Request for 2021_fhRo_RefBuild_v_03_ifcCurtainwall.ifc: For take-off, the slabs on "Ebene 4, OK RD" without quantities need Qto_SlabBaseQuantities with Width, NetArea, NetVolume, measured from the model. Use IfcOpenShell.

First a look at what the model holds.

```python
import ifcopenshell
import ifcopenshell.util.element
import ifcopenshell.util.unit

model = ifcopenshell.open("2021_fhRo_RefBuild_v_03_ifcCurtainwall.ifc")
print(model.schema)
for unit_type in ("LENGTHUNIT", "AREAUNIT", "VOLUMEUNIT"):
    print(unit_type, ifcopenshell.util.unit.calculate_unit_scale(model, unit_type))
storey = next(s for s in model.by_type("IfcBuildingStorey") if s.Name == "Ebene 4, OK RD")
slabs = [e for e in ifcopenshell.util.element.get_decomposition(storey) if e.is_a("IfcSlab")]
for e in sorted(slabs, key=lambda e: e.id()):
    print(e.id(), e.is_a(), e.Name, list(ifcopenshell.util.element.get_psets(e, qtos_only=True)), sep=" | ")
```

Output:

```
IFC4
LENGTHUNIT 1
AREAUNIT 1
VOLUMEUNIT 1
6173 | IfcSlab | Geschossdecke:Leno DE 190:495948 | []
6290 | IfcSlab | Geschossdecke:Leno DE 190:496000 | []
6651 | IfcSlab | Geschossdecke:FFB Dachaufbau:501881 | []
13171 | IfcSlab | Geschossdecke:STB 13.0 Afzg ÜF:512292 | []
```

```python
import ifcopenshell
import ifcopenshell.api.pset
import ifcopenshell.geom
import ifcopenshell.util.element
import ifcopenshell.util.shape
import ifcopenshell.util.unit

model = ifcopenshell.open("2021_fhRo_RefBuild_v_03_ifcCurtainwall.ifc")
unit_scale = ifcopenshell.util.unit.calculate_unit_scale(model)
area_scale = ifcopenshell.util.unit.calculate_unit_scale(model, "AREAUNIT")
volume_scale = ifcopenshell.util.unit.calculate_unit_scale(model, "VOLUMEUNIT")
settings = ifcopenshell.geom.settings()

storey = next(s for s in model.by_type("IfcBuildingStorey") if s.Name == "Ebene 4, OK RD")
slabs = [e for e in ifcopenshell.util.element.get_decomposition(storey) if e.is_a("IfcSlab")]

for e in sorted(slabs, key=lambda e: e.id()):
    if ifcopenshell.util.element.get_psets(e, qtos_only=True, should_inherit=False):
        continue
    # Geometry comes back in metres, in the element's own axes.
    shape = ifcopenshell.geom.create_shape(settings, e)
    values = {
        "Width": ifcopenshell.util.shape.get_z(shape.geometry) / unit_scale,
        "NetArea": ifcopenshell.util.shape.get_footprint_area(shape.geometry) / area_scale,
        "NetVolume": ifcopenshell.util.shape.get_volume(shape.geometry) / volume_scale,
    }
    qto = ifcopenshell.api.pset.add_qto(model, product=e, name="Qto_SlabBaseQuantities")
    ifcopenshell.api.pset.edit_qto(model, qto=qto, properties=values)
    print(e.id(), {k: round(v, 3) for k, v in values.items()})

model.write("2021_fhRo_RefBuild_v_03_ifcCurtainwall_edited.ifc")
```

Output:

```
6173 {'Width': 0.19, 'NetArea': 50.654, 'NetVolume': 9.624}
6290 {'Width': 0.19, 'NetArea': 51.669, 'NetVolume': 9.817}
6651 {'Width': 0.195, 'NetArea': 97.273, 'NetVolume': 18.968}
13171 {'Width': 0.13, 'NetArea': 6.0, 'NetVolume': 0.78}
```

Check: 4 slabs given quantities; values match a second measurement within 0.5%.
